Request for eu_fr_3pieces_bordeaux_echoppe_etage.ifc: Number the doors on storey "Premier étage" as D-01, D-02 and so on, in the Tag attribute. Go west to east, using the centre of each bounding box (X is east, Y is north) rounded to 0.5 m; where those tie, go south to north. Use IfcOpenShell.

First a look at what the model holds.

```python
import ifcopenshell
import ifcopenshell.util.element
import ifcopenshell.util.placement

model = ifcopenshell.open("eu_fr_3pieces_bordeaux_echoppe_etage.ifc")
print(model.schema)
storey = next(s for s in model.by_type("IfcBuildingStorey") if s.Name == "Premier étage")
doors = [e for e in ifcopenshell.util.element.get_decomposition(storey) if e.is_a("IfcDoor")]
for e in sorted(doors, key=lambda e: e.id()):
    origin = ifcopenshell.util.placement.get_local_placement(e.ObjectPlacement)[:3, 3]
    print(e.id(), e.Tag, e.Name, origin.round(2) + 0.0, sep=" | ")
```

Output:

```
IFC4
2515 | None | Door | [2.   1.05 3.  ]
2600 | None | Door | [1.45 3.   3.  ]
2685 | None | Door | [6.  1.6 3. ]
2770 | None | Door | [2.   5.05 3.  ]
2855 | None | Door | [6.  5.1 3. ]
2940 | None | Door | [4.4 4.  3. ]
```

```python
import ifcopenshell
import ifcopenshell.geom
import ifcopenshell.util.element
import ifcopenshell.util.shape

model = ifcopenshell.open("eu_fr_3pieces_bordeaux_echoppe_etage.ifc")
settings = ifcopenshell.geom.settings()
settings.set("use-world-coords", True)


def centre(element):
    shape = ifcopenshell.geom.create_shape(settings, element)
    return ifcopenshell.util.shape.get_bbox_centroid(shape.geometry)


storey = next(s for s in model.by_type("IfcBuildingStorey") if s.Name == "Premier étage")
doors = [e for e in ifcopenshell.util.element.get_decomposition(storey) if e.is_a("IfcDoor")]

# Insertion points can sit at a corner or the storey origin, so sort by the geometry (in metres).
centres = {e: centre(e) for e in doors}
doors.sort(key=lambda e: (round(centres[e][0] / 0.5), centres[e][1]))

for i, e in enumerate(doors, start=1):
    number = f"D-{i:02d}"
    e.Tag = number
    print(e.id(), number)

model.write("eu_fr_3pieces_bordeaux_echoppe_etage_edited.ifc")
```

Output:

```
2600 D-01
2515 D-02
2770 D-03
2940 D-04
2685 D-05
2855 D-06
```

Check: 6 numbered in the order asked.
